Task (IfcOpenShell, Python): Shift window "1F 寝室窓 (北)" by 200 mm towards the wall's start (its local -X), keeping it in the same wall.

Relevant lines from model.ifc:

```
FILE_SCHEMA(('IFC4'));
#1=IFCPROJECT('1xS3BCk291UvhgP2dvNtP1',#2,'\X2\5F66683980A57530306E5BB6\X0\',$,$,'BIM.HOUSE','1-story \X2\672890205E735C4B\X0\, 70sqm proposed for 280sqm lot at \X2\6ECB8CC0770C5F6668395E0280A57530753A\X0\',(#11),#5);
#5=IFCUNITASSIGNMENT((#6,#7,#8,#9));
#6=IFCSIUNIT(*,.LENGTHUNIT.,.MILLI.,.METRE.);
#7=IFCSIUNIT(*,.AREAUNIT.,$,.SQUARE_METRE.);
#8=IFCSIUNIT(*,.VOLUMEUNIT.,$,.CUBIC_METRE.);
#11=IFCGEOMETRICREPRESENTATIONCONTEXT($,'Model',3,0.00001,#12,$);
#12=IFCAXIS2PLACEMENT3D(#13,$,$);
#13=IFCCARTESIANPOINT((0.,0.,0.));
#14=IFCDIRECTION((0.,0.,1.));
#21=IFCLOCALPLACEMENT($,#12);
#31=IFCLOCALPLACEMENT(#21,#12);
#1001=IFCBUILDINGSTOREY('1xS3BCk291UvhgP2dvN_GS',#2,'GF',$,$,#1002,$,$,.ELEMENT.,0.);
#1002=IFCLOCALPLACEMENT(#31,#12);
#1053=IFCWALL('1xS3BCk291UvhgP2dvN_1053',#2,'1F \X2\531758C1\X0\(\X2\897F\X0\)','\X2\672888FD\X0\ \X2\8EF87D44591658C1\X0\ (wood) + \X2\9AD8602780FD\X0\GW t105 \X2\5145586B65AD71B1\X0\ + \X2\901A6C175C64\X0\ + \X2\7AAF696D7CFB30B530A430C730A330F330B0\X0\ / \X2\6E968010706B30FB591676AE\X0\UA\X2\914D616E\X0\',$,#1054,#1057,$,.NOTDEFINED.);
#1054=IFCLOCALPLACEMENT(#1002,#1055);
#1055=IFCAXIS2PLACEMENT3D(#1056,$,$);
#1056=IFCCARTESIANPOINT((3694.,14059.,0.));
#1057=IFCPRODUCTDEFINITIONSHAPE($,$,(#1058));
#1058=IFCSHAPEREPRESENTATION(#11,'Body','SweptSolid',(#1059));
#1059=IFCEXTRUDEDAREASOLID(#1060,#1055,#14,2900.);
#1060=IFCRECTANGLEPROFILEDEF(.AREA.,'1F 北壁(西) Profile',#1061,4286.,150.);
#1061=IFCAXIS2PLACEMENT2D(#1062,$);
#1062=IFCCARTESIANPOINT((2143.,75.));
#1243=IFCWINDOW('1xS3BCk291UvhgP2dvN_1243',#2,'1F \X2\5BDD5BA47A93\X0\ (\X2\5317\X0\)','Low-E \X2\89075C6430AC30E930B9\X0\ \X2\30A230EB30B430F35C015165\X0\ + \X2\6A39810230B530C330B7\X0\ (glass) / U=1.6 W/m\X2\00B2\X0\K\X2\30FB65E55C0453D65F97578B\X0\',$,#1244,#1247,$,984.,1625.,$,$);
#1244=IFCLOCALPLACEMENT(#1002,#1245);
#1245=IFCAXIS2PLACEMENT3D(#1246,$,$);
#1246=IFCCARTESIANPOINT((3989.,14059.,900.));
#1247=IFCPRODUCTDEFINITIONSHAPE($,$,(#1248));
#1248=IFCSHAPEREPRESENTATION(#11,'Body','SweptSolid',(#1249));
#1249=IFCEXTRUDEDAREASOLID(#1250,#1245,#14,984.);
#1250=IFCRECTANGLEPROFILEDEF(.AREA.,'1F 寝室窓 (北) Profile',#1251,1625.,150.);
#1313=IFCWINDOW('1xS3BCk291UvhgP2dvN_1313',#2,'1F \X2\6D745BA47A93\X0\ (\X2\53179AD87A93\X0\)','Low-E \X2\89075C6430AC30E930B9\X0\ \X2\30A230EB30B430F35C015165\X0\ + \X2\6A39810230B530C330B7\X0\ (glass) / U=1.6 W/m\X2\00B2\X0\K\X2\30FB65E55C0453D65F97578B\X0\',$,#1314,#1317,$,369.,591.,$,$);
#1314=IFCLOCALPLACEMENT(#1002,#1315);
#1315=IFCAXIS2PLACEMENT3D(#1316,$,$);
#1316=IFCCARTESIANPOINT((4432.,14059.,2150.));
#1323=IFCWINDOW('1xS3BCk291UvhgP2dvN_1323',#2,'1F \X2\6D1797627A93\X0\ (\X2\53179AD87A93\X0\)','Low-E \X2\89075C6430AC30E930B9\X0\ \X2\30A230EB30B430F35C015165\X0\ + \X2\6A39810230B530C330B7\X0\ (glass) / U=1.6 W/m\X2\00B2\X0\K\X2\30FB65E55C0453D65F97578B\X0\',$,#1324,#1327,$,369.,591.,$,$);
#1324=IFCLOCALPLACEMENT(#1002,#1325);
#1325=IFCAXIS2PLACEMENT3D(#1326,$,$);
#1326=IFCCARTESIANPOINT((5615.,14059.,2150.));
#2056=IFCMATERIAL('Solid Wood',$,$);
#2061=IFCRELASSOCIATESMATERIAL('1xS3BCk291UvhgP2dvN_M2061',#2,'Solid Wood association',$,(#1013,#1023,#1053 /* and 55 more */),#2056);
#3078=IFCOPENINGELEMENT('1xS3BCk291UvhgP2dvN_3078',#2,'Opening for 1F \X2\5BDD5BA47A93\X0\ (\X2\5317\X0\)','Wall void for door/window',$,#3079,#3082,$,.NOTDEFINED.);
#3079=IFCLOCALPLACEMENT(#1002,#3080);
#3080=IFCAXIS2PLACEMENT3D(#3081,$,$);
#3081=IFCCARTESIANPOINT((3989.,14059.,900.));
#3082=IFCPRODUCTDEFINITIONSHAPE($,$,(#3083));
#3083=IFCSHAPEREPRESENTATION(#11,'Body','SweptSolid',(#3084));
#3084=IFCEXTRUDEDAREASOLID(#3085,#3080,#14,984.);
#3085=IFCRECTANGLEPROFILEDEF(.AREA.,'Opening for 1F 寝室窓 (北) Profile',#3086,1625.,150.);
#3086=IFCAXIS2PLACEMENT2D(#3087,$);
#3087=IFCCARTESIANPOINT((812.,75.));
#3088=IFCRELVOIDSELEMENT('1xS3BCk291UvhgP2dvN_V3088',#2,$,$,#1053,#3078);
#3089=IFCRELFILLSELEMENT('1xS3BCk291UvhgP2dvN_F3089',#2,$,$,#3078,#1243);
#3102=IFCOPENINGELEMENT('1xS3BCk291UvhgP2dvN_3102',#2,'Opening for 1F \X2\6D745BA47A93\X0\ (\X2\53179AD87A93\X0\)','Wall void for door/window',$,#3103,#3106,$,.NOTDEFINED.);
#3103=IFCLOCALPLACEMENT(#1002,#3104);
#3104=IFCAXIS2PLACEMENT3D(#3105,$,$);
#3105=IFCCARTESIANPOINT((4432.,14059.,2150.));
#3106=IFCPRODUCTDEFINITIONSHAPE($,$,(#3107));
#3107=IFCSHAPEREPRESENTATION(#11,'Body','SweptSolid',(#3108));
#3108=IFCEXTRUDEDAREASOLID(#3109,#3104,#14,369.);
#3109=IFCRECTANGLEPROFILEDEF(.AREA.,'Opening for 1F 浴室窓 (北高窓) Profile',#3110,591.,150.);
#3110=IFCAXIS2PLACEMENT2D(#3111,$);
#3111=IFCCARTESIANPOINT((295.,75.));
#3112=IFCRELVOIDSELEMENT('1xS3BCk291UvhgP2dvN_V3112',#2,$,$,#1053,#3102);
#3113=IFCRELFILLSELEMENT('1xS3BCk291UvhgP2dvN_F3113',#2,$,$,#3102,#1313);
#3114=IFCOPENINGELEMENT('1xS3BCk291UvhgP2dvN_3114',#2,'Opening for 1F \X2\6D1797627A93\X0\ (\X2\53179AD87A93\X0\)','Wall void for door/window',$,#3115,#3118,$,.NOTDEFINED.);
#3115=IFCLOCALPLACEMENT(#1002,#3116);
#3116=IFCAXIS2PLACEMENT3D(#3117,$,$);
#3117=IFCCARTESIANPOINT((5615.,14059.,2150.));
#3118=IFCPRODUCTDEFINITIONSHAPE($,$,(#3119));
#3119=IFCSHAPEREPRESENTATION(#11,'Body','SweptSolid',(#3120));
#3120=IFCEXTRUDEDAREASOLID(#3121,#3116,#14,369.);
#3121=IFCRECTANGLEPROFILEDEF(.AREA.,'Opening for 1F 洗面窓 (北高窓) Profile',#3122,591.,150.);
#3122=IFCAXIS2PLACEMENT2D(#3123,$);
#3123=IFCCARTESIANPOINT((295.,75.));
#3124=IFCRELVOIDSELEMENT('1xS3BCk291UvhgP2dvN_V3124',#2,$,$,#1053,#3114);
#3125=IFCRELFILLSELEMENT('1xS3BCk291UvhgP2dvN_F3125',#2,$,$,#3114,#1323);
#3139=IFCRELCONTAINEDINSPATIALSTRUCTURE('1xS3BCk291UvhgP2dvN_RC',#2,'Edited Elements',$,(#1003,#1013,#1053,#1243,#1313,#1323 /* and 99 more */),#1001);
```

```python
import ifcopenshell
import ifcopenshell.api.geometry
import ifcopenshell.util.placement

model = ifcopenshell.open("model.ifc")

window = model.by_id(1243)
opening = window.FillsVoids[0].RelatingOpeningElement
wall = opening.VoidsElements[0].RelatingBuildingElement

wall_matrix = ifcopenshell.util.placement.get_local_placement(wall.ObjectPlacement)
shift = wall_matrix[:3, 0] * -200.0
before = ifcopenshell.util.placement.get_local_placement(window.ObjectPlacement)[:3, 3].copy()

# The window is not placed relative to its opening, so move both.
for product in (opening, window):
    matrix = ifcopenshell.util.placement.get_local_placement(product.ObjectPlacement)
    matrix[:3, 3] += shift
    ifcopenshell.api.geometry.edit_object_placement(model, product=product, matrix=matrix, is_si=False)

after = ifcopenshell.util.placement.get_local_placement(window.ObjectPlacement)[:3, 3]
print("window moved by", (after - before).round(3) + 0.0)

model.write("model_updated.ifc")
```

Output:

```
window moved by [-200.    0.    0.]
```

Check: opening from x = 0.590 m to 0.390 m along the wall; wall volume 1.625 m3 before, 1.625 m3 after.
